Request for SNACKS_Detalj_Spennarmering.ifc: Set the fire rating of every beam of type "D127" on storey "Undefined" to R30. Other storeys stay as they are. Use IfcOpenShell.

First a look at what the model holds.

```python
import ifcopenshell
import ifcopenshell.util.element

model = ifcopenshell.open("SNACKS_Detalj_Spennarmering.ifc")
print(model.schema)
storey = next(s for s in model.by_type("IfcBuildingStorey") if s.Name == "Undefined")
beams = [e for e in ifcopenshell.util.element.get_decomposition(storey) if e.is_a("IfcBeam")]
seen = {}
for e in beams:
    element_type = ifcopenshell.util.element.get_type(e)
    key = (element_type.Name if element_type != e and element_type else None, ifcopenshell.util.element.get_pset(e, "Pset_BeamCommon", "FireRating"))
    seen[key] = seen.get(key, 0) + 1
for (name, value), count in sorted(seen.items(), key=str):
    print(count, "x", name, "|", value)
```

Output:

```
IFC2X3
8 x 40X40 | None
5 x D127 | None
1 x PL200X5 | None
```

```python
import ifcopenshell
import ifcopenshell.api.pset
import ifcopenshell.util.element

model = ifcopenshell.open("SNACKS_Detalj_Spennarmering.ifc")

storey = next(s for s in model.by_type("IfcBuildingStorey") if s.Name == "Undefined")
beams = [e for e in ifcopenshell.util.element.get_decomposition(storey) if e.is_a("IfcBeam")]

count = 0
for e in beams:
    element_type = ifcopenshell.util.element.get_type(e)
    if element_type in (None, e) or element_type.Name != "D127":
        continue
    # add_pset returns the element's existing set when there is one.
    pset = ifcopenshell.api.pset.add_pset(model, product=e, name="Pset_BeamCommon")
    ifcopenshell.api.pset.edit_pset(model, pset=pset, properties={"FireRating": "R30"})
    count += 1

print(count, "beams updated")

model.write("SNACKS_Detalj_Spennarmering_updated.ifc")
```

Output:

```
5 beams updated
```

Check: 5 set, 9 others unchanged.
